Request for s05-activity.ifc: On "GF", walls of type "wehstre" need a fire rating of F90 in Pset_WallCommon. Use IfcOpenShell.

First a look at what the model holds.

```python
import ifcopenshell
import ifcopenshell.util.element

model = ifcopenshell.open("s05-activity.ifc")
print(model.schema)
storey = next(s for s in model.by_type("IfcBuildingStorey") if s.Name == "GF")
walls = [e for e in ifcopenshell.util.element.get_decomposition(storey) if e.is_a("IfcWall")]
seen = {}
for e in walls:
    element_type = ifcopenshell.util.element.get_type(e)
    key = (element_type.Name if element_type != e and element_type else None, ifcopenshell.util.element.get_pset(e, "Pset_WallCommon", "FireRating"))
    seen[key] = seen.get(key, 0) + 1
for (name, value), count in sorted(seen.items(), key=str):
    print(count, "x", name, "|", value)
```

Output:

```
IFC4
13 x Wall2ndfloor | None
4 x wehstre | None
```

```python
import ifcopenshell
import ifcopenshell.api.pset
import ifcopenshell.util.element

model = ifcopenshell.open("s05-activity.ifc")

storey = next(s for s in model.by_type("IfcBuildingStorey") if s.Name == "GF")
walls = [e for e in ifcopenshell.util.element.get_decomposition(storey) if e.is_a("IfcWall")]

count = 0
for e in walls:
    element_type = ifcopenshell.util.element.get_type(e)
    if element_type in (None, e) or element_type.Name != "wehstre":
        continue
    # add_pset returns the element's existing set when there is one.
    pset = ifcopenshell.api.pset.add_pset(model, product=e, name="Pset_WallCommon")
    ifcopenshell.api.pset.edit_pset(model, pset=pset, properties={"FireRating": "F90"})
    count += 1

print(count, "walls updated")

model.write("s05-activity-out.ifc")
```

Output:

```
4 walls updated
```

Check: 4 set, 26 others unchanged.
